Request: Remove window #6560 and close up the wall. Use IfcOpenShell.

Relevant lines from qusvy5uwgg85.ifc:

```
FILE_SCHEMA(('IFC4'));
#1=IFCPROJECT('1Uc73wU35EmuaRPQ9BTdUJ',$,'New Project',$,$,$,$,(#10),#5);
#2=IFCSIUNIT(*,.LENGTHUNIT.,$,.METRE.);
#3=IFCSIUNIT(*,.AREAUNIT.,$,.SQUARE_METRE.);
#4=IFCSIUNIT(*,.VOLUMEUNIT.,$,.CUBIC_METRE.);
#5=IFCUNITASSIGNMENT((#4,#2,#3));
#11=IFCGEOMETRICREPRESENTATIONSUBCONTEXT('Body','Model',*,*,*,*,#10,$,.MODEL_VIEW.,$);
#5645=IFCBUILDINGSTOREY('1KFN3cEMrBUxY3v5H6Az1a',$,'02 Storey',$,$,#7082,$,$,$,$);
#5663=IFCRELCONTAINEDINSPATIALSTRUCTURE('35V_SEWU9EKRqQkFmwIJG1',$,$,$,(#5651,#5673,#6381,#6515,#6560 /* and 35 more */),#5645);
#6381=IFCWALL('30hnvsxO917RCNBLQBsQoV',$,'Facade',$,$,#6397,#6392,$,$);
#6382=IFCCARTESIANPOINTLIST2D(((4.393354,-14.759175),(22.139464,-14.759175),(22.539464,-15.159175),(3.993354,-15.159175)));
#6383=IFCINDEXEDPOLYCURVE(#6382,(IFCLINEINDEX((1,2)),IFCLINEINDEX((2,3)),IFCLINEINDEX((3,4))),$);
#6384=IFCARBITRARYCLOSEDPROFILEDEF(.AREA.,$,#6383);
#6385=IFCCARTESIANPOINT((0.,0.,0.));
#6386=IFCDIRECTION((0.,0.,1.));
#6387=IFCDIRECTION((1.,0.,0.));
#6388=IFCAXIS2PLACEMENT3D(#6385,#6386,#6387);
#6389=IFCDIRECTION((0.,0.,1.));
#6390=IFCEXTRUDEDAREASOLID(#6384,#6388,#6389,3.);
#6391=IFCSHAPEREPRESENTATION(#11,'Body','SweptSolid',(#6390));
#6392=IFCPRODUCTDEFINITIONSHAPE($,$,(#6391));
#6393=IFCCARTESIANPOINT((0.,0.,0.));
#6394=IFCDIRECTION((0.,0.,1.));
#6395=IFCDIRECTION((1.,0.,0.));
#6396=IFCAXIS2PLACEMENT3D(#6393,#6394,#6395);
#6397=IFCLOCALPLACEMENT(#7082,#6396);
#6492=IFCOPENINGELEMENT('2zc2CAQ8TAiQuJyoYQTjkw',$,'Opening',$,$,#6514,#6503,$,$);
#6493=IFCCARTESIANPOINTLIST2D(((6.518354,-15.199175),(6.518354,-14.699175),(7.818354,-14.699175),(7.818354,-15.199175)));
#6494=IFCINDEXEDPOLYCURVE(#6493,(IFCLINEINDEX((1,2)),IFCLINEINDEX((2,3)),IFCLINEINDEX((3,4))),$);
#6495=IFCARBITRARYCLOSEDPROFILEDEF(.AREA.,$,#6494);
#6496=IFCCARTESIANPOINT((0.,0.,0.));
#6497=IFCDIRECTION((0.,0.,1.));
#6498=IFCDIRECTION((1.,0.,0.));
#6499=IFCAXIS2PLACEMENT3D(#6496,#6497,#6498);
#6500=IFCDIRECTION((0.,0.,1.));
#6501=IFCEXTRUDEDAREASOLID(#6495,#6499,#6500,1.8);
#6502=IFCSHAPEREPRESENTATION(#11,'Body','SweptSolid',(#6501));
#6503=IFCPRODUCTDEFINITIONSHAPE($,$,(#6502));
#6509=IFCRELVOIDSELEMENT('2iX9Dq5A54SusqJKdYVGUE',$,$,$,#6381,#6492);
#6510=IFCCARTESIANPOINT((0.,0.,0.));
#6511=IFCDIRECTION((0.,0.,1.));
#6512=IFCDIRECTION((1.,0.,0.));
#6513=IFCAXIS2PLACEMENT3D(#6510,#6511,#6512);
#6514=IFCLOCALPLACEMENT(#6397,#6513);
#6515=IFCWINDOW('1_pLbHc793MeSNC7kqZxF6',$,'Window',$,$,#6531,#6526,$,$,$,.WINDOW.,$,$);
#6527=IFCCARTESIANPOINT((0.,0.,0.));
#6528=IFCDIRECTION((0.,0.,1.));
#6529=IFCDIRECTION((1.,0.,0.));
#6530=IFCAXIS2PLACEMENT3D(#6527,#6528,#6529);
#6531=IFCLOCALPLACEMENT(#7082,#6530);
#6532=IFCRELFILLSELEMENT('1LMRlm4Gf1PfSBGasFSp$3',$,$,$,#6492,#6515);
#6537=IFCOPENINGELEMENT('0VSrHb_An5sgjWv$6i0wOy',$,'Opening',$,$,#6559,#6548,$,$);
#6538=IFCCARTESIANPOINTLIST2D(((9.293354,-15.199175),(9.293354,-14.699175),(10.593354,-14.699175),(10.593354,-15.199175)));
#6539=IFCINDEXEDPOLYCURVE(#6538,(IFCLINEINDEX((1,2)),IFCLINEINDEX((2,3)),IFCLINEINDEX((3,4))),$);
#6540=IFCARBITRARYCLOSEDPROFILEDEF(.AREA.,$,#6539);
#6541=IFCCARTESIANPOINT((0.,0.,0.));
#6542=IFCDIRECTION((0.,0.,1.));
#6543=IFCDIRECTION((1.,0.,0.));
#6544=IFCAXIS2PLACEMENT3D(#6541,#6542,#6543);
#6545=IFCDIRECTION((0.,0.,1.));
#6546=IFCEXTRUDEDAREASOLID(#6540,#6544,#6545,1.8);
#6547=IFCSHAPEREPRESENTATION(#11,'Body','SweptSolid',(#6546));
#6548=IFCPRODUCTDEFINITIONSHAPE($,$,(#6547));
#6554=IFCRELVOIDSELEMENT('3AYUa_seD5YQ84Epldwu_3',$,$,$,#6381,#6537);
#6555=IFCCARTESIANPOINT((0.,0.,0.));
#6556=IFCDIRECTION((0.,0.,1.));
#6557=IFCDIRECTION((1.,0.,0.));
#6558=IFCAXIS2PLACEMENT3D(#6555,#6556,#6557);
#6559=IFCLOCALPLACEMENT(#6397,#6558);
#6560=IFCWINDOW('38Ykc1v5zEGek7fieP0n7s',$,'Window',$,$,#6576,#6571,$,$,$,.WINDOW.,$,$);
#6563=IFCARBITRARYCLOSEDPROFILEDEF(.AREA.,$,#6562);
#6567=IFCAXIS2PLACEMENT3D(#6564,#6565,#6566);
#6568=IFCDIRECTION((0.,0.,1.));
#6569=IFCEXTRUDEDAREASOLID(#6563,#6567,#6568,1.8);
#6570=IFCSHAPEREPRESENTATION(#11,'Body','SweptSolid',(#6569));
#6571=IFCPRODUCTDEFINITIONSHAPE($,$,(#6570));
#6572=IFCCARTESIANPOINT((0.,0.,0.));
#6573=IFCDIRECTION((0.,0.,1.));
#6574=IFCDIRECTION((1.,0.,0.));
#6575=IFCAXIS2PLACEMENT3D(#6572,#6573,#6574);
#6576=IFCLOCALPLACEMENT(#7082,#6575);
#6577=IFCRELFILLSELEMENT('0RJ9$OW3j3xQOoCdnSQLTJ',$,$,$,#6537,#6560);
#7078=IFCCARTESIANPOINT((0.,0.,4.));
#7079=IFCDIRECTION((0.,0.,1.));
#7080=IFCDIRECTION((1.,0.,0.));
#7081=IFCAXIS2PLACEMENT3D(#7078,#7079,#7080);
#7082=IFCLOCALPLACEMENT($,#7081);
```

```python
import ifcopenshell
import ifcopenshell.api.feature
import ifcopenshell.api.root
import ifcopenshell.geom
import ifcopenshell.util.shape

model = ifcopenshell.open("qusvy5uwgg85.ifc")
settings = ifcopenshell.geom.settings()


def volume(element):
    """Net volume in cubic metres, openings subtracted."""
    shape = ifcopenshell.geom.create_shape(settings, element)
    return ifcopenshell.util.shape.get_volume(shape.geometry)


window = model.by_id(6560)
opening = window.FillsVoids[0].RelatingOpeningElement
wall = opening.VoidsElements[0].RelatingBuildingElement
before = volume(wall)

ifcopenshell.api.root.remove_product(model, product=window)
ifcopenshell.api.feature.remove_feature(model, feature=opening)

after = volume(wall)

print(f"wall volume {before:.3f} -> {after:.3f} m3")

model.write("qusvy5uwgg85_v2.ifc")
```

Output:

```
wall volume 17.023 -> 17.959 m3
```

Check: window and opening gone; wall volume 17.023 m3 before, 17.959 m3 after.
